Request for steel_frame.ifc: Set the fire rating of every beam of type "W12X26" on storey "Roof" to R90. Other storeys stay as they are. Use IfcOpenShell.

First a look at what the model holds.

```python
import ifcopenshell
import ifcopenshell.util.element

model = ifcopenshell.open("steel_frame.ifc")
print(model.schema)
storey = next(s for s in model.by_type("IfcBuildingStorey") if s.Name == "Roof")
beams = [e for e in ifcopenshell.util.element.get_decomposition(storey) if e.is_a("IfcBeam")]
seen = {}
for e in beams:
    element_type = ifcopenshell.util.element.get_type(e)
    key = (element_type.Name if element_type != e and element_type else None, ifcopenshell.util.element.get_pset(e, "Pset_BeamCommon", "FireRating"))
    seen[key] = seen.get(key, 0) + 1
for (name, value), count in sorted(seen.items(), key=str):
    print(count, "x", name, "|", value)
```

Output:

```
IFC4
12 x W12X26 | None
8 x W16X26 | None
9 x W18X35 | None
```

```python
import ifcopenshell
import ifcopenshell.api.pset
import ifcopenshell.util.element

model = ifcopenshell.open("steel_frame.ifc")

storey = next(s for s in model.by_type("IfcBuildingStorey") if s.Name == "Roof")
beams = [e for e in ifcopenshell.util.element.get_decomposition(storey) if e.is_a("IfcBeam")]

count = 0
for e in beams:
    element_type = ifcopenshell.util.element.get_type(e)
    if element_type in (None, e) or element_type.Name != "W12X26":
        continue
    # add_pset returns the element's existing set when there is one.
    pset = ifcopenshell.api.pset.add_pset(model, product=e, name="Pset_BeamCommon")
    ifcopenshell.api.pset.edit_pset(model, pset=pset, properties={"FireRating": "R90"})
    count += 1

print(count, "beams updated")

model.write("steel_frame_v2.ifc")
```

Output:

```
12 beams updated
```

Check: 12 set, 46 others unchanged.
